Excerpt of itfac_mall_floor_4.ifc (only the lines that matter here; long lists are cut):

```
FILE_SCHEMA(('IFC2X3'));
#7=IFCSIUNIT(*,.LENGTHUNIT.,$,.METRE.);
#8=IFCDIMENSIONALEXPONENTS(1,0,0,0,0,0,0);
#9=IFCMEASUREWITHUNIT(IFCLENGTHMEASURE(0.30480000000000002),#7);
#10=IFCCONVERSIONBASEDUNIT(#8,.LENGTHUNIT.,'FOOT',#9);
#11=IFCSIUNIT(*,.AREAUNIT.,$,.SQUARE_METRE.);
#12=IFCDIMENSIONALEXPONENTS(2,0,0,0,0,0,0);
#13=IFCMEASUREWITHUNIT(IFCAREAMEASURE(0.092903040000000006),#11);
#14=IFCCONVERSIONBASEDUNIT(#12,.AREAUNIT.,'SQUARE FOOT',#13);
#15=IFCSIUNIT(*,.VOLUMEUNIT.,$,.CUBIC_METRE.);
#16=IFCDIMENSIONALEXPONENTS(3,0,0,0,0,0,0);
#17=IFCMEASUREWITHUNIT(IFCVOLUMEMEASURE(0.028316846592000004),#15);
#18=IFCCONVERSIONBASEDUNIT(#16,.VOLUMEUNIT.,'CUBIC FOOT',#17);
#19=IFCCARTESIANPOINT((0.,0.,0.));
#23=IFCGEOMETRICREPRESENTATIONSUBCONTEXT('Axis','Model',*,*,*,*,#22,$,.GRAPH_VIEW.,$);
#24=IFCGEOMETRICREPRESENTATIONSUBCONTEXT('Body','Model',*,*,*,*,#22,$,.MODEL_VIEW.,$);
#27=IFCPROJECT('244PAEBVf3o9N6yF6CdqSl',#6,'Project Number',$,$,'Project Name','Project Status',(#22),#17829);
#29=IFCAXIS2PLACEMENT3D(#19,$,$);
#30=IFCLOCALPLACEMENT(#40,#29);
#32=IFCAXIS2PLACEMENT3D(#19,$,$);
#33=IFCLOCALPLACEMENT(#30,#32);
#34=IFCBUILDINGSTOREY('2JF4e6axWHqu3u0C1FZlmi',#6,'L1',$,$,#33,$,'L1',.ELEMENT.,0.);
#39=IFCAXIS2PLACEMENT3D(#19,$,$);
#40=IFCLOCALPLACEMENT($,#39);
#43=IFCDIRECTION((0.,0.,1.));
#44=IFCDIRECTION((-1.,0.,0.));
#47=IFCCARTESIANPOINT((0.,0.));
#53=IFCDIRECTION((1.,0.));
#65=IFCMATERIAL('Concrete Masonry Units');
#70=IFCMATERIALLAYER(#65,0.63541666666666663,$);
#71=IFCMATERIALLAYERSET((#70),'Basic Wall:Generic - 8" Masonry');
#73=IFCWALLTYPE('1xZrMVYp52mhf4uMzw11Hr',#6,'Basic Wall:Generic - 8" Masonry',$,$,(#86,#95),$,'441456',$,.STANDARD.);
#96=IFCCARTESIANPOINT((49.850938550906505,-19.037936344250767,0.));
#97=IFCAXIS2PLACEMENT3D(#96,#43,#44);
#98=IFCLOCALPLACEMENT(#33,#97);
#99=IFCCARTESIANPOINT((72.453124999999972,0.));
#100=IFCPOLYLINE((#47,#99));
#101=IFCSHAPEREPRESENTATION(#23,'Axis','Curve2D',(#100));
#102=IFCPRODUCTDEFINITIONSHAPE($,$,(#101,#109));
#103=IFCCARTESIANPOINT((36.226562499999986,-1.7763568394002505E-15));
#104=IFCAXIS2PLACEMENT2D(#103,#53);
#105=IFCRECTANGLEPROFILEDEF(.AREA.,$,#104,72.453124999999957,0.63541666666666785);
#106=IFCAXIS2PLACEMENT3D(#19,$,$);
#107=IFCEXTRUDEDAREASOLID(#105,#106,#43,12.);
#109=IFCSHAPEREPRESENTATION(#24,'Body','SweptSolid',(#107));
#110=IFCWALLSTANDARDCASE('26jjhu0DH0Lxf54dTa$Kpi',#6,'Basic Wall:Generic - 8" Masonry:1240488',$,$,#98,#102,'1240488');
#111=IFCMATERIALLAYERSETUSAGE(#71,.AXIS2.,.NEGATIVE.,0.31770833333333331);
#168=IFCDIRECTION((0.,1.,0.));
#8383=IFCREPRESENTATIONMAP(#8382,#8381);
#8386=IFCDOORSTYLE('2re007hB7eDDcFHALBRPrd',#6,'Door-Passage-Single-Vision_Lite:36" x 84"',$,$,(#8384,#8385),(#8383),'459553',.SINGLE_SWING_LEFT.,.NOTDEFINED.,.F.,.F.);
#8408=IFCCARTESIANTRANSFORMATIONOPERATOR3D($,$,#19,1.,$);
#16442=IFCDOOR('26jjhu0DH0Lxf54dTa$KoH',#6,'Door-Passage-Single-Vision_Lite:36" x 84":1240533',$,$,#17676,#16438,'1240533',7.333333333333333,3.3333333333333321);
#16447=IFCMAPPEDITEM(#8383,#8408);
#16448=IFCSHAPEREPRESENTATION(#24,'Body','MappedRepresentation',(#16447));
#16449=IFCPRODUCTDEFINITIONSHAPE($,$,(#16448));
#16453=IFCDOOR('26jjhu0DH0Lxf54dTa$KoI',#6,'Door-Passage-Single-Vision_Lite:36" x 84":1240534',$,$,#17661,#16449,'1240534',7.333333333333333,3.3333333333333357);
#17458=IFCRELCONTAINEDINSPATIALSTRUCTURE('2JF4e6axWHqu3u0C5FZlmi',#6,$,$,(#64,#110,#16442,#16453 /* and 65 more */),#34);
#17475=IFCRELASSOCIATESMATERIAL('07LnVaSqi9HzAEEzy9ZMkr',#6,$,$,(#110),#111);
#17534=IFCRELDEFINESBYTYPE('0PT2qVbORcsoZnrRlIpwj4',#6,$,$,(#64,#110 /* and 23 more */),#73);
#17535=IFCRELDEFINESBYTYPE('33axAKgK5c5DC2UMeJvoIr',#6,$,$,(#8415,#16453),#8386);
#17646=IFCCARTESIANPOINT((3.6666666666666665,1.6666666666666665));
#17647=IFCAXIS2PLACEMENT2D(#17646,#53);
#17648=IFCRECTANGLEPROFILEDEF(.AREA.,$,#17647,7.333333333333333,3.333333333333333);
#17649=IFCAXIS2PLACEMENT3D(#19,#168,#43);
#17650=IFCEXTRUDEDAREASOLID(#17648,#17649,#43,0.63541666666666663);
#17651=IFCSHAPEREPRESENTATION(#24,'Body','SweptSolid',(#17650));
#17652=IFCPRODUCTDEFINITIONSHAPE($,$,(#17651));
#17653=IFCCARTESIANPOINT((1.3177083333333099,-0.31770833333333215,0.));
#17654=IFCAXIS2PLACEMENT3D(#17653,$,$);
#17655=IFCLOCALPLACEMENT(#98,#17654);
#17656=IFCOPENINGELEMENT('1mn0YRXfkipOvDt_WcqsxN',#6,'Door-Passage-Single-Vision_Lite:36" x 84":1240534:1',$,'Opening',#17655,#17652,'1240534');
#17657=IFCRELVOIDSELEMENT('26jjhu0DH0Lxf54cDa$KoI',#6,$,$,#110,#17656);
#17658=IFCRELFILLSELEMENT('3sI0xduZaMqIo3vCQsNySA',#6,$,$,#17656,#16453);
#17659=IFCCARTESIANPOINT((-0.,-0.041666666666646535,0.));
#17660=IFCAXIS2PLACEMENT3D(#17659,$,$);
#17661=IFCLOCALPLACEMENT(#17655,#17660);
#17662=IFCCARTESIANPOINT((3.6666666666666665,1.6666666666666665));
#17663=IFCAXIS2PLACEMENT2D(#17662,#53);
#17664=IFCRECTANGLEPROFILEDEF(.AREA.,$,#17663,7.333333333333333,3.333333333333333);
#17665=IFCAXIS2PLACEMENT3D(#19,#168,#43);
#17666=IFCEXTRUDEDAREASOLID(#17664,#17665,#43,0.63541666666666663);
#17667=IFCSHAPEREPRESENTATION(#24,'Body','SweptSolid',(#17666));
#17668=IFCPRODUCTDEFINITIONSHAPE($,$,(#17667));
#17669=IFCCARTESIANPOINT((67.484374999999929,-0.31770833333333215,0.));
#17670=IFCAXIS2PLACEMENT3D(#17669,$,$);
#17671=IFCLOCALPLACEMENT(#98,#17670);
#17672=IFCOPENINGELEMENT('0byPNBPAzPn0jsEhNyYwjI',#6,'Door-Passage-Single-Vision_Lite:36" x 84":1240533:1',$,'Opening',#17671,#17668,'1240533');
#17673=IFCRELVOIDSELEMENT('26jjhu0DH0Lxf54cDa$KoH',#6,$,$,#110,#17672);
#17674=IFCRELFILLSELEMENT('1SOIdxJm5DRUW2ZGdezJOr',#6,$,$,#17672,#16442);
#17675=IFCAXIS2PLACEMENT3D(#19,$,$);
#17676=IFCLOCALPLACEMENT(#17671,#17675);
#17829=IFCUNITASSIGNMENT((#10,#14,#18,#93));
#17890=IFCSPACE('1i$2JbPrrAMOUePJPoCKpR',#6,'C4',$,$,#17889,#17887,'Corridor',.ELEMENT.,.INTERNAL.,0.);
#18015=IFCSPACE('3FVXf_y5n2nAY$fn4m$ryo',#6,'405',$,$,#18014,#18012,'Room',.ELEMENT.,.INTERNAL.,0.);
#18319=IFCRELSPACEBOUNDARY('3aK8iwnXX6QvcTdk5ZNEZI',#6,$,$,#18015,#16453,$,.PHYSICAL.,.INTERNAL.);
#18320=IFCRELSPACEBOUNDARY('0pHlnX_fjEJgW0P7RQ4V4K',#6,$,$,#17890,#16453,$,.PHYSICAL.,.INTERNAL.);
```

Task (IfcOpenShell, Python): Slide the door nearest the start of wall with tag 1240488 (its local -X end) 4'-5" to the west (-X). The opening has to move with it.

```python
import ifcopenshell
import ifcopenshell.api.geometry
import ifcopenshell.util.placement
import ifcopenshell.util.unit

model = ifcopenshell.open("itfac_mall_floor_4.ifc")
unit_scale = ifcopenshell.util.unit.calculate_unit_scale(model)

door = model.by_guid("26jjhu0DH0Lxf54dTa$KoI")
opening = door.FillsVoids[0].RelatingOpeningElement
wall = opening.VoidsElements[0].RelatingBuildingElement

wall_matrix = ifcopenshell.util.placement.get_local_placement(wall.ObjectPlacement)
shift = wall_matrix[:3, 0] * 53 * 0.0254 / unit_scale
before = ifcopenshell.util.placement.get_local_placement(door.ObjectPlacement)[:3, 3].copy()

# The door is placed relative to its opening, so it follows when the opening moves.
matrix = ifcopenshell.util.placement.get_local_placement(opening.ObjectPlacement)
matrix[:3, 3] += shift
ifcopenshell.api.geometry.edit_object_placement(
    model, product=opening, matrix=matrix, is_si=False, should_transform_children=True
)

after = ifcopenshell.util.placement.get_local_placement(door.ObjectPlacement)[:3, 3]
print("door moved by", (after - before).round(3) + 0.0)

model.write("itfac_mall_floor_4_rev.ifc")
```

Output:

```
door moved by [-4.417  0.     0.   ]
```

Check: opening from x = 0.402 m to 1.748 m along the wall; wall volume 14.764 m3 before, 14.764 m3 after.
